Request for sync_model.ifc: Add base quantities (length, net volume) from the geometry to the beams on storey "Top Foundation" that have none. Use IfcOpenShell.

First a look at what the model holds.

```python
import ifcopenshell
import ifcopenshell.util.element
import ifcopenshell.util.unit

model = ifcopenshell.open("sync_model.ifc")
print(model.schema)
for unit_type in ("LENGTHUNIT", "AREAUNIT", "VOLUMEUNIT"):
    print(unit_type, ifcopenshell.util.unit.calculate_unit_scale(model, unit_type))
storey = next(s for s in model.by_type("IfcBuildingStorey") if s.Name == "Top Foundation")
beams = [e for e in ifcopenshell.util.element.get_decomposition(storey) if e.is_a("IfcBeam")]
for e in sorted(beams, key=lambda e: e.id()):
    print(e.id(), e.is_a(), e.Name, list(ifcopenshell.util.element.get_psets(e, qtos_only=True)), sep=" | ")
```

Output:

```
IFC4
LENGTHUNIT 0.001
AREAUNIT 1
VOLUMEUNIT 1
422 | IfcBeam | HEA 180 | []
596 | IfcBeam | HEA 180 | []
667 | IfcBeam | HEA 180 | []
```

```python
import ifcopenshell
import ifcopenshell.api.pset
import ifcopenshell.geom
import ifcopenshell.util.element
import ifcopenshell.util.shape
import ifcopenshell.util.unit

model = ifcopenshell.open("sync_model.ifc")
unit_scale = ifcopenshell.util.unit.calculate_unit_scale(model)
volume_scale = ifcopenshell.util.unit.calculate_unit_scale(model, "VOLUMEUNIT")
settings = ifcopenshell.geom.settings()

storey = next(s for s in model.by_type("IfcBuildingStorey") if s.Name == "Top Foundation")
beams = [e for e in ifcopenshell.util.element.get_decomposition(storey) if e.is_a("IfcBeam")]

for e in sorted(beams, key=lambda e: e.id()):
    if ifcopenshell.util.element.get_psets(e, qtos_only=True, should_inherit=False):
        continue
    # Geometry comes back in metres, in the element's own axes.
    shape = ifcopenshell.geom.create_shape(settings, e)
    values = {
        "Length": ifcopenshell.util.shape.get_max_xyz(shape.geometry) / unit_scale,
        "NetVolume": ifcopenshell.util.shape.get_volume(shape.geometry) / volume_scale,
    }
    qto = ifcopenshell.api.pset.add_qto(model, product=e, name="Qto_BeamBaseQuantities")
    ifcopenshell.api.pset.edit_qto(model, qto=qto, properties=values)
    print(e.id(), {k: round(v, 3) for k, v in values.items()})

model.write("sync_model_edited.ifc")
```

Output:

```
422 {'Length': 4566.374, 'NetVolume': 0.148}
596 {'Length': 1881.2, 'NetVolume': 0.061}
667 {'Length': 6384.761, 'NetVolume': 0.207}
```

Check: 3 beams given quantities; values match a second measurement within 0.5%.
